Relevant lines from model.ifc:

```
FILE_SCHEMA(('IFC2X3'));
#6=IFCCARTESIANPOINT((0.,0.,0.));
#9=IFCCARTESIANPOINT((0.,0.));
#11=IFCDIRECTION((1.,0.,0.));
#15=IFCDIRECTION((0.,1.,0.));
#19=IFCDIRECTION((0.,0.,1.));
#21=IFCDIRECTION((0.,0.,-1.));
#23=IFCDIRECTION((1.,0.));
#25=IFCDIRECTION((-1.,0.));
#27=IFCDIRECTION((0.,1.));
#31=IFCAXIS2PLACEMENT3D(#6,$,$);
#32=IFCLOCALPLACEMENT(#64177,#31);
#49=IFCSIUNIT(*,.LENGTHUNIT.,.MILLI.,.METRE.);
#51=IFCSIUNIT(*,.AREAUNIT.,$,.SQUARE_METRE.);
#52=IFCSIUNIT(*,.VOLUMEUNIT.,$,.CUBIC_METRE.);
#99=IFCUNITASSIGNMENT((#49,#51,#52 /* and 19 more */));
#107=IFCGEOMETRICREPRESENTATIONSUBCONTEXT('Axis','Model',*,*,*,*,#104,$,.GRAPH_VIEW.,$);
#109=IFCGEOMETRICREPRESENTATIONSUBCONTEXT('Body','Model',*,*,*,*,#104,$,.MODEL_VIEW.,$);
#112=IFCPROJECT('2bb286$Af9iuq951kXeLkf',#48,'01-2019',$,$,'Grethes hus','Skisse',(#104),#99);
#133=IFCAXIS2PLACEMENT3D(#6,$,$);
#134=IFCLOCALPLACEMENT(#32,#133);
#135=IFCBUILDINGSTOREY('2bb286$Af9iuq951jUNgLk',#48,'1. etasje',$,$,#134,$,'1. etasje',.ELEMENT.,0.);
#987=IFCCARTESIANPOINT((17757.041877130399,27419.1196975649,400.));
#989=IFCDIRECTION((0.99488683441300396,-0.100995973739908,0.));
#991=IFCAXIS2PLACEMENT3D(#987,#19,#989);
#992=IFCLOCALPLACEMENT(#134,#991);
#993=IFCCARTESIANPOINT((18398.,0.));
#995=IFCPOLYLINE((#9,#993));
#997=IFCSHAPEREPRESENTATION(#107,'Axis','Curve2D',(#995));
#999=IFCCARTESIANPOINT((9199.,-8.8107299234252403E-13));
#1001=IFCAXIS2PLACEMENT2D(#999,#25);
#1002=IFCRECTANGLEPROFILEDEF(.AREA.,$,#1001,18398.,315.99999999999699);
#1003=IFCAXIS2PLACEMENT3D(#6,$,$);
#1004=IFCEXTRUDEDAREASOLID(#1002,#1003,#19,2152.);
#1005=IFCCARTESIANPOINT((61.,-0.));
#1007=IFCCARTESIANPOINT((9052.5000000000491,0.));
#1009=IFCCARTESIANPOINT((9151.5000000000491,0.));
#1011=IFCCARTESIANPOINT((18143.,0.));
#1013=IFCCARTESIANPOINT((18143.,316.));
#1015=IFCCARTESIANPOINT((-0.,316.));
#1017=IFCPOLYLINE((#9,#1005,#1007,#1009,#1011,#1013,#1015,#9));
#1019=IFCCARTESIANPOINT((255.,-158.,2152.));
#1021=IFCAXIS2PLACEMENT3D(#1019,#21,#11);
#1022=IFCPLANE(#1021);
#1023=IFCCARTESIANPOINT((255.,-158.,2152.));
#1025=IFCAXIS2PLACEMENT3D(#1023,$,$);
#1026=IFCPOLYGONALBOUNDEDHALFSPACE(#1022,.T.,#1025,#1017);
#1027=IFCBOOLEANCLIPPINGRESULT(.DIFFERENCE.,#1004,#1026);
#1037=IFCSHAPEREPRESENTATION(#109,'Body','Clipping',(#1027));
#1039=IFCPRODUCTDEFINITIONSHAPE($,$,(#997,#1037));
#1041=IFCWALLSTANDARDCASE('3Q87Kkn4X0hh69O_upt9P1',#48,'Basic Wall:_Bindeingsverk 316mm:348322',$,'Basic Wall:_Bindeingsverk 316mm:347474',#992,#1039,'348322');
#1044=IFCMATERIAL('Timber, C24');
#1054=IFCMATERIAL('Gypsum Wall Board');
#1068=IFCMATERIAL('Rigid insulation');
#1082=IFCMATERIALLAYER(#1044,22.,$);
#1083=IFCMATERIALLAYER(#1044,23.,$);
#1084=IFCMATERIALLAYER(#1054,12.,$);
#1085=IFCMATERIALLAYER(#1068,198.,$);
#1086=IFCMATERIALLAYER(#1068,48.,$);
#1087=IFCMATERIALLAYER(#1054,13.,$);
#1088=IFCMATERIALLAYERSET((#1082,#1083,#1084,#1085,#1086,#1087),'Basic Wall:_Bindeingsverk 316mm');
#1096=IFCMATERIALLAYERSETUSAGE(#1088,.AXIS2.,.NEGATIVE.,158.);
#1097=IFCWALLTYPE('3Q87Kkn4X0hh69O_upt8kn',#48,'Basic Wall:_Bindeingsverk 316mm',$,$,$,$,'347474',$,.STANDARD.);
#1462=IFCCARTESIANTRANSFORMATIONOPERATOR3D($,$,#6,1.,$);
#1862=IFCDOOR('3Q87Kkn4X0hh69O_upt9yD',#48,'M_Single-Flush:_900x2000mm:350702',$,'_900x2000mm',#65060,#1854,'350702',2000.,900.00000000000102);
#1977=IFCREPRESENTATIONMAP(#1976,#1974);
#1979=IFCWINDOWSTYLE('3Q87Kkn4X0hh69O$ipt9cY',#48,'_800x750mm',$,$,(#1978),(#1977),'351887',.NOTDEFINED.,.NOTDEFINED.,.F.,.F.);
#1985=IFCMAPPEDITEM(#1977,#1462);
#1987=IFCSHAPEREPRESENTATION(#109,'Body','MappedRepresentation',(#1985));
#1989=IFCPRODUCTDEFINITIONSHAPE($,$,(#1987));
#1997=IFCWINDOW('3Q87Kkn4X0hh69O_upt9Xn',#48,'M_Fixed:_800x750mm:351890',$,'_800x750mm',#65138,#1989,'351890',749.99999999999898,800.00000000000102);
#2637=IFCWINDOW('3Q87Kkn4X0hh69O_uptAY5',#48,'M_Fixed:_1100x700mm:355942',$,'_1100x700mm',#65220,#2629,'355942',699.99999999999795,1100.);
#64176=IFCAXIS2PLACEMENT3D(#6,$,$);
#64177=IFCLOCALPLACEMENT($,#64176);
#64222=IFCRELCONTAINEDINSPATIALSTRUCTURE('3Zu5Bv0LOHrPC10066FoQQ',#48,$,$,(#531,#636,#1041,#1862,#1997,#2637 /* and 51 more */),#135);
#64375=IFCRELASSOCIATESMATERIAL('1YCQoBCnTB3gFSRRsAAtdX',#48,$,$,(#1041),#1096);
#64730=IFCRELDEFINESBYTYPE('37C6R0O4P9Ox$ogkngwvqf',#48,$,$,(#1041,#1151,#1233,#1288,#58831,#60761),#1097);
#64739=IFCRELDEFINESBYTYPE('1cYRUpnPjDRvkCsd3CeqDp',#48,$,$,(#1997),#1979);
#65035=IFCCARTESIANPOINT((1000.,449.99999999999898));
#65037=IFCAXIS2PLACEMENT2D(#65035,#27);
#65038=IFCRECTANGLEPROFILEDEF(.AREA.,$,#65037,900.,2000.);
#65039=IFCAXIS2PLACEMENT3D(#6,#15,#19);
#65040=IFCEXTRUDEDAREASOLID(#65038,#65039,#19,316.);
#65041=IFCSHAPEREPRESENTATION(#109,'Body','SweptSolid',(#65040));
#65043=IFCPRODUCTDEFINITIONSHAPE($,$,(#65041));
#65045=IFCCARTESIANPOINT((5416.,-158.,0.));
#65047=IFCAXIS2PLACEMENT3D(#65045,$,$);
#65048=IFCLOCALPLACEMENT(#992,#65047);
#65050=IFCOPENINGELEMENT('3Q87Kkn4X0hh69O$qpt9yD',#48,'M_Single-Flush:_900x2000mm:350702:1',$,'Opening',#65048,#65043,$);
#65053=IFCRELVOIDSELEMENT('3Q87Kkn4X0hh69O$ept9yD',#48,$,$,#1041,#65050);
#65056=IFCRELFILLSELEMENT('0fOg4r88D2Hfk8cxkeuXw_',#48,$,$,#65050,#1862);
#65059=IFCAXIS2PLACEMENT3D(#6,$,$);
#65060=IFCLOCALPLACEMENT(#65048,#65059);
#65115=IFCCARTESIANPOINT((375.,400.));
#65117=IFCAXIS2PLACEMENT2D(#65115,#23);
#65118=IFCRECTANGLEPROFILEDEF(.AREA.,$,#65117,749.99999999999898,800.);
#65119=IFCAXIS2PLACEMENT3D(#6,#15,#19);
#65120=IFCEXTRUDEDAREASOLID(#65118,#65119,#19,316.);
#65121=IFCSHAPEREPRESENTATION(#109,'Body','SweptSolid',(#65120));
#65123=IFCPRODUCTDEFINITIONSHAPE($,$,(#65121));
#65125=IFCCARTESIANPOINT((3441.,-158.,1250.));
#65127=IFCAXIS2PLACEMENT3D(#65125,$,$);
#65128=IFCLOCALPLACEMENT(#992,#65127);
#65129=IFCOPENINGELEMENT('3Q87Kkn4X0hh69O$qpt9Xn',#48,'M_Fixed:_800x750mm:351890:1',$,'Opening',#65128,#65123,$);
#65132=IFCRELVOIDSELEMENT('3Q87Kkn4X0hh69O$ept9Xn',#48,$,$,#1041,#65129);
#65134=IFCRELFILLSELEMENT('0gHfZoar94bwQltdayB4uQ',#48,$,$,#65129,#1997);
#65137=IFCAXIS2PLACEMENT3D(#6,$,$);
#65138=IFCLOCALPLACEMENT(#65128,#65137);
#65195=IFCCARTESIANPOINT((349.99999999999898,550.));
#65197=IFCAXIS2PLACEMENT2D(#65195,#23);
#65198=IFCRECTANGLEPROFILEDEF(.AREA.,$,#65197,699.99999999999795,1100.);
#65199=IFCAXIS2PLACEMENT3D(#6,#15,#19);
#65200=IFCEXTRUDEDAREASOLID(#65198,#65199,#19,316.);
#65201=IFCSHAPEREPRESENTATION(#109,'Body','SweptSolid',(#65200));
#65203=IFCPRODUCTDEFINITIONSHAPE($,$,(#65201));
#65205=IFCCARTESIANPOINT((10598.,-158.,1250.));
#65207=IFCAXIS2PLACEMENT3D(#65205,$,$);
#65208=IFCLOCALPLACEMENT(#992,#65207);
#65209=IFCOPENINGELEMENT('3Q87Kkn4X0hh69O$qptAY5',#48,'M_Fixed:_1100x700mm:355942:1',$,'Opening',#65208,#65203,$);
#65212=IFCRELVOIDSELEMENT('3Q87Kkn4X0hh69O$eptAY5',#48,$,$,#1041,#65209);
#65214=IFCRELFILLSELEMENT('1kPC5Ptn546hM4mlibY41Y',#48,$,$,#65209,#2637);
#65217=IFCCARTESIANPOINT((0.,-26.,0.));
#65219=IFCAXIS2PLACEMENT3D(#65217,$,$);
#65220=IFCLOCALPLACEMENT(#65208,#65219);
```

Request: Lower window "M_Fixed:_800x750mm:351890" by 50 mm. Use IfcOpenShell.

```python
import numpy as np
import ifcopenshell
import ifcopenshell.api.geometry
import ifcopenshell.util.placement
import ifcopenshell.util.unit

model = ifcopenshell.open("model.ifc")
unit_scale = ifcopenshell.util.unit.calculate_unit_scale(model)

window = model.by_guid("3Q87Kkn4X0hh69O_upt9Xn")
opening = window.FillsVoids[0].RelatingOpeningElement
dz = -0.05 / unit_scale

shift = np.array([0.0, 0.0, dz])
# The window is placed relative to its opening, so it follows when the opening moves.
matrix = ifcopenshell.util.placement.get_local_placement(opening.ObjectPlacement)
matrix[:3, 3] += shift
ifcopenshell.api.geometry.edit_object_placement(
    model, product=opening, matrix=matrix, is_si=False, should_transform_children=True
)

print(f"moved by {dz * unit_scale:+.3f} m")

model.write("model_edited.ifc")
```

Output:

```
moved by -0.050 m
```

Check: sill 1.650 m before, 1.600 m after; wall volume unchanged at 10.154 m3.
